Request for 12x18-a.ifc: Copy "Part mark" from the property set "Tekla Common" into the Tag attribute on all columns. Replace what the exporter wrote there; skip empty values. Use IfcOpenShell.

First a look at what the model holds.

```python
import ifcopenshell
import ifcopenshell.util.element

model = ifcopenshell.open("12x18-a.ifc")
print(model.schema)
columns = model.by_type("IfcColumn")
print(len(columns), "columns")
for e in columns[:8]:
    source = ifcopenshell.util.element.get_pset(e, "Tekla Common", "Part mark")
    target = e.Tag
    print(e.id(), repr(source), repr(target), sep=" | ")
```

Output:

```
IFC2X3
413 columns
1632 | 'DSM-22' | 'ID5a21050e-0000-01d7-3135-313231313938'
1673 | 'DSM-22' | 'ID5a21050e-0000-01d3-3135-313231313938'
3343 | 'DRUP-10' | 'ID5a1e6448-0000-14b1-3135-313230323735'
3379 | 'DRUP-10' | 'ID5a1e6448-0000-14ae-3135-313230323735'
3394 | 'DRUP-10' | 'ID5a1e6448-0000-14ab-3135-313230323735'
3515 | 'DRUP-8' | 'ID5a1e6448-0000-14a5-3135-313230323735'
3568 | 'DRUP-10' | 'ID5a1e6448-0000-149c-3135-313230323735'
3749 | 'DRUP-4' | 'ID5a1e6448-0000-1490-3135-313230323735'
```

```python
import ifcopenshell
import ifcopenshell.util.element

model = ifcopenshell.open("12x18-a.ifc")

count = 0
for e in model.by_type("IfcColumn"):
    value = ifcopenshell.util.element.get_pset(e, "Tekla Common", "Part mark")
    current = e.Tag
    if not value or not value.strip() or current == value:
        continue
    e.Tag = value
    count += 1

print(count, "columns updated")

model.write("12x18-a_v2.ifc")
```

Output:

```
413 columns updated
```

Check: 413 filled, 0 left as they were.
